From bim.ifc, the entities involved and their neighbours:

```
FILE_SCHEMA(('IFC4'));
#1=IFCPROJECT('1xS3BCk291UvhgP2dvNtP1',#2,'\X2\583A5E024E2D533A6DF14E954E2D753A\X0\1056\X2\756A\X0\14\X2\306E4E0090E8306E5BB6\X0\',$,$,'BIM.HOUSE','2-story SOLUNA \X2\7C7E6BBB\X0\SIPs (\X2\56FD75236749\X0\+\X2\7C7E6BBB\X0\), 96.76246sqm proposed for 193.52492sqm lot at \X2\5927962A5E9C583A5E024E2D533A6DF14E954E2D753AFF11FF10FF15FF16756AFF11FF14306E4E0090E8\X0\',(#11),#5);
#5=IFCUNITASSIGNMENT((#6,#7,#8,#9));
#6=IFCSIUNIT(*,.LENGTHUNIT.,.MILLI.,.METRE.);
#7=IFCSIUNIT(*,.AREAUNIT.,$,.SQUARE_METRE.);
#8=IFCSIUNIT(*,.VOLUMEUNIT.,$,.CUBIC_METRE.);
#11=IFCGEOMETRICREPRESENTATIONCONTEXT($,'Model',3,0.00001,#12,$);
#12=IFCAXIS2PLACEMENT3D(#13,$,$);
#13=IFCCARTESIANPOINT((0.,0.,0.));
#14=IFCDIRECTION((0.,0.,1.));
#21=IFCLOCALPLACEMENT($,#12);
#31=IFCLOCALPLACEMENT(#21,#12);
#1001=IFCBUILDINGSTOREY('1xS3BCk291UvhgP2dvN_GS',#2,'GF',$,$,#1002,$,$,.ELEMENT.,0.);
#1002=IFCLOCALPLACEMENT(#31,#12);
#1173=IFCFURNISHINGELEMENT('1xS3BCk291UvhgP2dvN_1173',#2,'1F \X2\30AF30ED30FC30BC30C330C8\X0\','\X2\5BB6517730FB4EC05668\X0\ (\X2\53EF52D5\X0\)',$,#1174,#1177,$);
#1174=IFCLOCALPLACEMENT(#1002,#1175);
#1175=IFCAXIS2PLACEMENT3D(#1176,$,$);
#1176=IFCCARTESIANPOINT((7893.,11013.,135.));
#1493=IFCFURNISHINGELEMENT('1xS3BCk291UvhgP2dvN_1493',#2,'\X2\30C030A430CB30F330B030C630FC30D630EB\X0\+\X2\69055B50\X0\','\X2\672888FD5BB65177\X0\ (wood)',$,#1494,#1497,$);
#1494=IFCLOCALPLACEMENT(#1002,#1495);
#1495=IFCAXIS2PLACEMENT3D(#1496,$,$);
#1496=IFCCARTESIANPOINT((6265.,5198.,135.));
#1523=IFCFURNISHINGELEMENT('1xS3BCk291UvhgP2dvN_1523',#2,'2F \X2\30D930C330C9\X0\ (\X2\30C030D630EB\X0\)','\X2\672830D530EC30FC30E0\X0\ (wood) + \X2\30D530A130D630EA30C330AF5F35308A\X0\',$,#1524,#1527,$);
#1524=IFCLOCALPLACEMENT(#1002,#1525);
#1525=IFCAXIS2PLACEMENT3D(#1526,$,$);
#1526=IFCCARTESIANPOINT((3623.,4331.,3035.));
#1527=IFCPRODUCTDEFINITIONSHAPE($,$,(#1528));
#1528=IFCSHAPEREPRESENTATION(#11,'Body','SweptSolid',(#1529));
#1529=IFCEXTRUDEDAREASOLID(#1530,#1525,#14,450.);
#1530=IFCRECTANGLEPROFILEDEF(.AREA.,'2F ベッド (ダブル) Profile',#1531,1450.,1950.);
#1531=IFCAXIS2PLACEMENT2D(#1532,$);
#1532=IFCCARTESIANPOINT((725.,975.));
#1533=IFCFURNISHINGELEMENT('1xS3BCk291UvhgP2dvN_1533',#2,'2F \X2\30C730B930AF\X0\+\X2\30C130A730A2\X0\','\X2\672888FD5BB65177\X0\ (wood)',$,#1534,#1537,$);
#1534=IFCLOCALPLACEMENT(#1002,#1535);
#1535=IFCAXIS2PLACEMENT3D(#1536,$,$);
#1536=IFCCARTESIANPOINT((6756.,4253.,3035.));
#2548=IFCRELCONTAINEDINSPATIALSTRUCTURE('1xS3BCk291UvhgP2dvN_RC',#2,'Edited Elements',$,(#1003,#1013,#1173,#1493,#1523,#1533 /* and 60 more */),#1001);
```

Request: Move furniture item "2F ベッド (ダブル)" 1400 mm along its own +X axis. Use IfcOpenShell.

```python
import ifcopenshell
import ifcopenshell.api.geometry
import ifcopenshell.util.placement

model = ifcopenshell.open("bim.ifc")

item = model.by_id(1523)
matrix = ifcopenshell.util.placement.get_local_placement(item.ObjectPlacement)
matrix[:3, 3] += matrix[:3, 0] * 1400.0
ifcopenshell.api.geometry.edit_object_placement(model, product=item, matrix=matrix, is_si=False)

print(ifcopenshell.util.placement.get_local_placement(item.ObjectPlacement).round(3) + 0.0)

model.write("bim_edited.ifc")
```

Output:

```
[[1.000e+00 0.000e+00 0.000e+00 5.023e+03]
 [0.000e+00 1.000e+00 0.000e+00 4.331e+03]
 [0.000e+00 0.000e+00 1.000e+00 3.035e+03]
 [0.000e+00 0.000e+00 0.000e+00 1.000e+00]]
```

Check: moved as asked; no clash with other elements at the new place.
